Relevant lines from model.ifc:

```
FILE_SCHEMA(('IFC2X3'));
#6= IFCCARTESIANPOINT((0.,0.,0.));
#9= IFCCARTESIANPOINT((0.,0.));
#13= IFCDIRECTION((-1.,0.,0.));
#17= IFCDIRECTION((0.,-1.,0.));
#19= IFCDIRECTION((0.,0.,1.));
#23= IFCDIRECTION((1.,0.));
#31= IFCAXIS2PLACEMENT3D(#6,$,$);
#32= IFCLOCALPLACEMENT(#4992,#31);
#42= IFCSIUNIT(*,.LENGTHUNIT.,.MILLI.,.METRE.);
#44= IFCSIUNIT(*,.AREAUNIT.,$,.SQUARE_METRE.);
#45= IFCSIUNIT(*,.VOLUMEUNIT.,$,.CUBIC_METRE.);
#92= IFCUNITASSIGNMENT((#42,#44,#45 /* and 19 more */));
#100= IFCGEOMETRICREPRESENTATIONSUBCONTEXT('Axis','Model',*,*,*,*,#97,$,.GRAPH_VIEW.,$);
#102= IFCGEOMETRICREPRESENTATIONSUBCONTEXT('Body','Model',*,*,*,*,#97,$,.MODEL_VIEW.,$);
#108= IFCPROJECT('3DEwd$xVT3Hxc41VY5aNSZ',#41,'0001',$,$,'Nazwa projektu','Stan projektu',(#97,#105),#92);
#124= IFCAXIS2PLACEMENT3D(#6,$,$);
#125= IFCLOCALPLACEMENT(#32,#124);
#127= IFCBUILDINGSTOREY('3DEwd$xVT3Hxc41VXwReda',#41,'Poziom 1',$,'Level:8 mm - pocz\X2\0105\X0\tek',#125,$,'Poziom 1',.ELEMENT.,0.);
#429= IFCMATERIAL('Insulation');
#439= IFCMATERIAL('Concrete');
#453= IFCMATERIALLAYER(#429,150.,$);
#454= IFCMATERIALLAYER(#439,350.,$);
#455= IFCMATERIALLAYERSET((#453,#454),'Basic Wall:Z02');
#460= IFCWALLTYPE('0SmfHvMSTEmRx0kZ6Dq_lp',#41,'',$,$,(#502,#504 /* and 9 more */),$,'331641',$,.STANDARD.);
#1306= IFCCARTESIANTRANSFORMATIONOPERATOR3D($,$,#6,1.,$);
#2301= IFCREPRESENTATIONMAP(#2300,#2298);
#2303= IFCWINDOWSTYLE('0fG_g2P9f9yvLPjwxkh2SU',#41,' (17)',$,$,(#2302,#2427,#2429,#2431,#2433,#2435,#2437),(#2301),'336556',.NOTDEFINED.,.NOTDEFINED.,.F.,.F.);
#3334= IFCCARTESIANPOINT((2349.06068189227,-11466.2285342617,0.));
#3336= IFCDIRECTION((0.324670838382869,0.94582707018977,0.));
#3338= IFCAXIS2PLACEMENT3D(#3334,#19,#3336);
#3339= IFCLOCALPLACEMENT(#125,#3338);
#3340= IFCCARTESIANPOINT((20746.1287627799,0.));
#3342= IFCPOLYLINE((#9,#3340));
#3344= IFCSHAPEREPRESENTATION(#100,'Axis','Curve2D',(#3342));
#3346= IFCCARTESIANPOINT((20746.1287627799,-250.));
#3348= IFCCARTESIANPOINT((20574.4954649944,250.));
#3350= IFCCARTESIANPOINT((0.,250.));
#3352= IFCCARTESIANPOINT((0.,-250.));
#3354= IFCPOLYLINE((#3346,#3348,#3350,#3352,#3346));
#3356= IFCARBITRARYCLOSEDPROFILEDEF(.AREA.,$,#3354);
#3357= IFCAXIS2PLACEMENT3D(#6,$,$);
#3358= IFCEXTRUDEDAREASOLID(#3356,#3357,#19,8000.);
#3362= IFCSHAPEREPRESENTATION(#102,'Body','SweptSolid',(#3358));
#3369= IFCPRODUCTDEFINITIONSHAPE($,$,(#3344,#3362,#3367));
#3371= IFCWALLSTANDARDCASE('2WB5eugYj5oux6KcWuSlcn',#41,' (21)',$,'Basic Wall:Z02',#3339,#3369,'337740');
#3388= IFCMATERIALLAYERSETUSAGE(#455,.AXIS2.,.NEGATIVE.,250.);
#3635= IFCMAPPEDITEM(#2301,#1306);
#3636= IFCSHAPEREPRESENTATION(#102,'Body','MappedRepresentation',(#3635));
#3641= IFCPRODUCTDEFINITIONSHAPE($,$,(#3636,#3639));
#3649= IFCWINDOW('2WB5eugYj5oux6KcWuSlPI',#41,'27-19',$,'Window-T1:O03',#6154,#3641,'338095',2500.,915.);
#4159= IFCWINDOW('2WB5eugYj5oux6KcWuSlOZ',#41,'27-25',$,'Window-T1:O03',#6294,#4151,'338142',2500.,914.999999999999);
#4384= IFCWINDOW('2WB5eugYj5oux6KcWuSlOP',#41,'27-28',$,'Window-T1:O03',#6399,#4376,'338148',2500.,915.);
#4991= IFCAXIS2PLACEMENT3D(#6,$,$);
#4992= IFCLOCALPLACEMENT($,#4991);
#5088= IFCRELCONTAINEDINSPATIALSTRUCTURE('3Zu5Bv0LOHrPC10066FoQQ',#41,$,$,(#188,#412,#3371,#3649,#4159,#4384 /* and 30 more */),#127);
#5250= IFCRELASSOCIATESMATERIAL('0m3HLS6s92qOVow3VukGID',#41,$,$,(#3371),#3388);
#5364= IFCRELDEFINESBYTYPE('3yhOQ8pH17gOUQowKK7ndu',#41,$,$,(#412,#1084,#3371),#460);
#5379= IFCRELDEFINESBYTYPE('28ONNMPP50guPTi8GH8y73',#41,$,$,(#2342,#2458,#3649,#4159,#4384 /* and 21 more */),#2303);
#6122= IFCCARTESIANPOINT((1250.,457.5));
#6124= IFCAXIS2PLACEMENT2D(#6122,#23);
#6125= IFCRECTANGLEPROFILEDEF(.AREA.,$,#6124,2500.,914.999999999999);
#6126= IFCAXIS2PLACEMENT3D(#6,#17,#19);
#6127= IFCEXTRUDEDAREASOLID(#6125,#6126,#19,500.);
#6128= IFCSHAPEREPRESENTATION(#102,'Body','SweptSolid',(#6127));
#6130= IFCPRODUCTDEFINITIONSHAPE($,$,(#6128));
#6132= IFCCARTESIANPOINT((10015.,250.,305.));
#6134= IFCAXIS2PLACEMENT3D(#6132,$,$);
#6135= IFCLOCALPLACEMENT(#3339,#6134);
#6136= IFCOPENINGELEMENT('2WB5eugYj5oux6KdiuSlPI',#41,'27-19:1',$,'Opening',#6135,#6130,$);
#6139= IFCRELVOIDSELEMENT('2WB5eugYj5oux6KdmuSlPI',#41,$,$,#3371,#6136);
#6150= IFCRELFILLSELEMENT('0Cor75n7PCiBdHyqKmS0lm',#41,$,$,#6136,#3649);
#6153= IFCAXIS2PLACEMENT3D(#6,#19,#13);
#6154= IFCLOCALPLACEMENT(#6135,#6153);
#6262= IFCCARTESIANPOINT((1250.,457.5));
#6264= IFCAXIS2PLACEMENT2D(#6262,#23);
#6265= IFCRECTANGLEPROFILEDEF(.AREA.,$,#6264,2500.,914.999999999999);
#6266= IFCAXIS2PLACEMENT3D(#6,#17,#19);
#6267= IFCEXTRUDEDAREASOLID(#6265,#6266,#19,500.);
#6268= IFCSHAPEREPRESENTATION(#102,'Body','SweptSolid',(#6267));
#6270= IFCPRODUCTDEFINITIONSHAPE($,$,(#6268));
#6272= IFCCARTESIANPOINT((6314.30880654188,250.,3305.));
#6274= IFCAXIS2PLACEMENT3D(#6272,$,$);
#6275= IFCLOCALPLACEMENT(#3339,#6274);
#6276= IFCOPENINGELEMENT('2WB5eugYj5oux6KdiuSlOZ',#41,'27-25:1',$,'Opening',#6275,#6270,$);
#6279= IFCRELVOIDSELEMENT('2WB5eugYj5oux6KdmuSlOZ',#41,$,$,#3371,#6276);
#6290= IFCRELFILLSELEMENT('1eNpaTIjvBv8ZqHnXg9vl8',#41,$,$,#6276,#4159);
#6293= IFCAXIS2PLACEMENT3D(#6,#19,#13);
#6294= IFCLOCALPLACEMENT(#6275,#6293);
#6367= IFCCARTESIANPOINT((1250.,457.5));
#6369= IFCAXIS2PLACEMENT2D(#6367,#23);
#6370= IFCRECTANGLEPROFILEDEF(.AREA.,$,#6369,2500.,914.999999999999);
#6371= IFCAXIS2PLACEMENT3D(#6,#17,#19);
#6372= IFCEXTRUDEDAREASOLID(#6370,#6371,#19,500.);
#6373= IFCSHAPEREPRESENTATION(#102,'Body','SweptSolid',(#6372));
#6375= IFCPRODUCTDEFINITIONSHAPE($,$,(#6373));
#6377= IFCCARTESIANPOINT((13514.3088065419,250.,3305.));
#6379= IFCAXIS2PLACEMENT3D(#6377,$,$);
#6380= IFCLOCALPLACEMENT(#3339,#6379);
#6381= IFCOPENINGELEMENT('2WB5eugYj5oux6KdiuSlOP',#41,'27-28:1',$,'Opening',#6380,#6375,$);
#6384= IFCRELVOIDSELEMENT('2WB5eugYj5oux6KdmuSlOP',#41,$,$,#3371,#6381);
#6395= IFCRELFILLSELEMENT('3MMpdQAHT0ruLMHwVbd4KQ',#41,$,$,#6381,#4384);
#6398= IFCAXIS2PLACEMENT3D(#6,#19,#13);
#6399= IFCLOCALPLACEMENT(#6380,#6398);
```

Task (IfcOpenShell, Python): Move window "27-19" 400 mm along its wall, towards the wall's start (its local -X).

```python
import ifcopenshell
import ifcopenshell.api.geometry
import ifcopenshell.util.placement

model = ifcopenshell.open("model.ifc")

window = model.by_guid("2WB5eugYj5oux6KcWuSlPI")
opening = window.FillsVoids[0].RelatingOpeningElement
wall = opening.VoidsElements[0].RelatingBuildingElement

wall_matrix = ifcopenshell.util.placement.get_local_placement(wall.ObjectPlacement)
shift = wall_matrix[:3, 0] * -400.0
before = ifcopenshell.util.placement.get_local_placement(window.ObjectPlacement)[:3, 3].copy()

# The window is placed relative to its opening, so it follows when the opening moves.
matrix = ifcopenshell.util.placement.get_local_placement(opening.ObjectPlacement)
matrix[:3, 3] += shift
ifcopenshell.api.geometry.edit_object_placement(
    model, product=opening, matrix=matrix, is_si=False, should_transform_children=True
)

after = ifcopenshell.util.placement.get_local_placement(window.ObjectPlacement)[:3, 3]
print("window moved by", (after - before).round(3) + 0.0)

model.write("model_v2.ifc")
```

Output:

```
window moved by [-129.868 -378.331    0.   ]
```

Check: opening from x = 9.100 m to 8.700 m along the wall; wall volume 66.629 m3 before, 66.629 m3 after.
